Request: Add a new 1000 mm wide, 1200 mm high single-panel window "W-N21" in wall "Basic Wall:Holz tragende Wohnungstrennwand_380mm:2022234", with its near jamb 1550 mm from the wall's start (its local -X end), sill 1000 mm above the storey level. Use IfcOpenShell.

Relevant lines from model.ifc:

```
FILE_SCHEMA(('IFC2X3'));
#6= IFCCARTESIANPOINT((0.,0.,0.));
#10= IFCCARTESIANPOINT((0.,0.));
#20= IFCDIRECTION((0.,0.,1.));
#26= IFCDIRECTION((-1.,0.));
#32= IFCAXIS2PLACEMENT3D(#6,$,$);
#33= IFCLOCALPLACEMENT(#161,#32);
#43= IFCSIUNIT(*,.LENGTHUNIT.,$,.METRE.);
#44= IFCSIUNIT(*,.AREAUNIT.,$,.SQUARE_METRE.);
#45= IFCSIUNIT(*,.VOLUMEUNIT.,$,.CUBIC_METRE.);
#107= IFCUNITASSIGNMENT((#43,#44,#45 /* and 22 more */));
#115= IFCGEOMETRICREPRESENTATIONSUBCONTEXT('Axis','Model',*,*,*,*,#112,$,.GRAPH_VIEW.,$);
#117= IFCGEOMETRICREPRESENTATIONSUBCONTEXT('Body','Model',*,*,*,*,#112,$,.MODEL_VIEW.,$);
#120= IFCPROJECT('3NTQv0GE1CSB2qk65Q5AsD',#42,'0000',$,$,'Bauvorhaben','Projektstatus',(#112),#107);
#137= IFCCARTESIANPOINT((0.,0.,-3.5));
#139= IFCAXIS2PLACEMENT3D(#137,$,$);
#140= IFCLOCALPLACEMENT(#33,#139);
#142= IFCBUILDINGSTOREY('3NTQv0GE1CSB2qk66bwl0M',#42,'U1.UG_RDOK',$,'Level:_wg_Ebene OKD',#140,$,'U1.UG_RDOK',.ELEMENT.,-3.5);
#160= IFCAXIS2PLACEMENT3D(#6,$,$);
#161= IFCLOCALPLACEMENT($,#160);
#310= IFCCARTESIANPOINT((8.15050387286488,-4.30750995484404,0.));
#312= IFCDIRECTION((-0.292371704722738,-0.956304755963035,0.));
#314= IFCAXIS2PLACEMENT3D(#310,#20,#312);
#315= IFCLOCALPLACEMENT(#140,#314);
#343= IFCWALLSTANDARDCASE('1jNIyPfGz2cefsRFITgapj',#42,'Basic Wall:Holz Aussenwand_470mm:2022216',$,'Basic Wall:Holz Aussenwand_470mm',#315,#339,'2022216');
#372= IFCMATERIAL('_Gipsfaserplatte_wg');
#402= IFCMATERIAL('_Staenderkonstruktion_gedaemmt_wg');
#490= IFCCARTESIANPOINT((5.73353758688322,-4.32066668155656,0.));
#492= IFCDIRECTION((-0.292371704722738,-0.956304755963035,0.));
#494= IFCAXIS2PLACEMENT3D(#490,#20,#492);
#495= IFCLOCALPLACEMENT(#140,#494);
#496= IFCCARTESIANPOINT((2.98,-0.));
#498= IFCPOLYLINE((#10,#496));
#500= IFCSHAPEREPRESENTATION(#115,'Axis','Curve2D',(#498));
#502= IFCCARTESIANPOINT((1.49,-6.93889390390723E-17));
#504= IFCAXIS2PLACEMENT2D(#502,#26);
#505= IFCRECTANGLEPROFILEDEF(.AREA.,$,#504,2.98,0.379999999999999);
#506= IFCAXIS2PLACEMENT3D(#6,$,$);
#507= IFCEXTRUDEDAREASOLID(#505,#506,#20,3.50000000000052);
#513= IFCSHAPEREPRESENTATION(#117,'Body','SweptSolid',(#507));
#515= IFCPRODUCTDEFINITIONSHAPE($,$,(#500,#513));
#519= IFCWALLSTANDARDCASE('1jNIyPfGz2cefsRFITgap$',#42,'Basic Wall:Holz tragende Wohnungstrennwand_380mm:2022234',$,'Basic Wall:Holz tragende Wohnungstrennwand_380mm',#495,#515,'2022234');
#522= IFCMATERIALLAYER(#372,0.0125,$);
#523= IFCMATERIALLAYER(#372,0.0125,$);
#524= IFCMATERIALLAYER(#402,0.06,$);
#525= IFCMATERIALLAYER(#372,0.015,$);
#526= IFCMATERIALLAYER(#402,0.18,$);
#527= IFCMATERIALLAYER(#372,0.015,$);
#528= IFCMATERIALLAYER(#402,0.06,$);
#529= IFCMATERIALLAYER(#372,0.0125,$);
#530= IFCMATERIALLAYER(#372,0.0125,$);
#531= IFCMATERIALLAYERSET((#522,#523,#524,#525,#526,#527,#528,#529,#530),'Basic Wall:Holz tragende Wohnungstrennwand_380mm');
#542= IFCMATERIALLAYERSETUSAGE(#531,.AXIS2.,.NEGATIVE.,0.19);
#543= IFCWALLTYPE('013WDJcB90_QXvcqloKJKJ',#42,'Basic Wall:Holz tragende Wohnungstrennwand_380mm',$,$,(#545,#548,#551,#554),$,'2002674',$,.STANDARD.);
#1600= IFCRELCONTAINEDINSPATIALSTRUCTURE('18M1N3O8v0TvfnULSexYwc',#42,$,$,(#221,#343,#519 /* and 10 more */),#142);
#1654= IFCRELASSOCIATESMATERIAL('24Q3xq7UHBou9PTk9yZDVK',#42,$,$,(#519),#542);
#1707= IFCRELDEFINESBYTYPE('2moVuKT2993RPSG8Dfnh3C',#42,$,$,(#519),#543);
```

```python
import numpy as np
import ifcopenshell
import ifcopenshell.api.feature
import ifcopenshell.api.geometry
import ifcopenshell.api.root
import ifcopenshell.api.spatial
import ifcopenshell.api.type
import ifcopenshell.geom
import ifcopenshell.util.element
import ifcopenshell.util.placement
import ifcopenshell.util.representation
import ifcopenshell.util.shape
import ifcopenshell.util.unit

model = ifcopenshell.open("model.ifc")
unit_scale = ifcopenshell.util.unit.calculate_unit_scale(model)
settings = ifcopenshell.geom.settings()


def volume(element):
    """Net volume in cubic metres, openings subtracted."""
    shape = ifcopenshell.geom.create_shape(settings, element)
    return ifcopenshell.util.shape.get_volume(shape.geometry)


wall = model.by_guid("1jNIyPfGz2cefsRFITgap$")
storey = ifcopenshell.util.element.get_container(wall, ifc_class="IfcBuildingStorey")
context = ifcopenshell.util.representation.get_context(model, "Model", "Body", "MODEL_VIEW")
before = volume(wall)

width, height, from_end, sill = 1, 1.2, 1.55, 1  # metres

# The wall runs along its own X axis, and the end named is its -X end.
wall_shape = ifcopenshell.geom.create_shape(settings, wall)
x, y, z = ifcopenshell.util.shape.get_vertices(wall_shape.geometry).T
start = x.min() + from_end
face, thickness = float(y.min()), float(y.max() - y.min())
wall_matrix = ifcopenshell.util.placement.get_local_placement(wall.ObjectPlacement)
level = ifcopenshell.util.placement.get_local_placement(storey.ObjectPlacement)[2, 3]


def in_wall(x, y):
    """Placement at x, y metres in the wall's axes, at sill height."""
    matrix = wall_matrix.copy()
    matrix[:, 3] = wall_matrix @ np.array([x / unit_scale, y / unit_scale, 0.0, 1.0])
    matrix[2, 3] = level + sill / unit_scale
    return matrix


# Opening: a box that overshoots both wall faces by 50 mm.
opening = ifcopenshell.api.root.create_entity(model, ifc_class="IfcOpeningElement")
box = ifcopenshell.api.geometry.add_wall_representation(
    model, context=context, length=width, height=height, thickness=thickness + 0.1
)
ifcopenshell.api.geometry.assign_representation(model, product=opening, representation=box)
ifcopenshell.api.geometry.edit_object_placement(model, product=opening, matrix=in_wall(start, face - 0.05), is_si=False)
ifcopenshell.api.feature.add_feature(model, feature=opening, element=wall)

window = ifcopenshell.api.root.create_entity(model, ifc_class="IfcWindow", name="W-N21")
window.OverallWidth, window.OverallHeight = width / unit_scale, height / unit_scale
body = ifcopenshell.api.geometry.add_window_representation(
    model,
    context=context,
    overall_width=window.OverallWidth,
    overall_height=window.OverallHeight,
    partition_type="SINGLE_PANEL",
)
ifcopenshell.api.geometry.assign_representation(model, product=window, representation=body)
ifcopenshell.api.spatial.assign_container(model, products=[window], relating_structure=storey)
fills = ifcopenshell.api.feature.add_filling(model, opening=opening, element=window)
fills.OwnerHistory = window.OwnerHistory  # required in IFC2X3

# IFC2X3 keeps the operation on the window style.
style = ifcopenshell.api.root.create_entity(model, ifc_class="IfcWindowStyle", name="W-N21")
style.OperationType, style.ConstructionType = "SINGLE_PANEL", "NOTDEFINED"
style.ParameterTakesPrecedence = style.Sizeable = False
ifcopenshell.api.type.assign_type(model, related_objects=[window], relating_type=style)

# Centre the window in the wall's thickness.
ifcopenshell.api.geometry.edit_object_placement(model, product=window, matrix=in_wall(start, face), is_si=False)
window_shape = ifcopenshell.geom.create_shape(settings, window)
depth = ifcopenshell.util.shape.get_vertices(window_shape.geometry)[:, 1]
offset = face + thickness / 2 - (depth.min() + depth.max()) / 2
ifcopenshell.api.geometry.edit_object_placement(model, product=window, matrix=in_wall(start, offset), is_si=False)

after = volume(wall)

print(f"wall volume {before:.3f} -> {after:.3f} m3")

model.write("model-out.ifc")
```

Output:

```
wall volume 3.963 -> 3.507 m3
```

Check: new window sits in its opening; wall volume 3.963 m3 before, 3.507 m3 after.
